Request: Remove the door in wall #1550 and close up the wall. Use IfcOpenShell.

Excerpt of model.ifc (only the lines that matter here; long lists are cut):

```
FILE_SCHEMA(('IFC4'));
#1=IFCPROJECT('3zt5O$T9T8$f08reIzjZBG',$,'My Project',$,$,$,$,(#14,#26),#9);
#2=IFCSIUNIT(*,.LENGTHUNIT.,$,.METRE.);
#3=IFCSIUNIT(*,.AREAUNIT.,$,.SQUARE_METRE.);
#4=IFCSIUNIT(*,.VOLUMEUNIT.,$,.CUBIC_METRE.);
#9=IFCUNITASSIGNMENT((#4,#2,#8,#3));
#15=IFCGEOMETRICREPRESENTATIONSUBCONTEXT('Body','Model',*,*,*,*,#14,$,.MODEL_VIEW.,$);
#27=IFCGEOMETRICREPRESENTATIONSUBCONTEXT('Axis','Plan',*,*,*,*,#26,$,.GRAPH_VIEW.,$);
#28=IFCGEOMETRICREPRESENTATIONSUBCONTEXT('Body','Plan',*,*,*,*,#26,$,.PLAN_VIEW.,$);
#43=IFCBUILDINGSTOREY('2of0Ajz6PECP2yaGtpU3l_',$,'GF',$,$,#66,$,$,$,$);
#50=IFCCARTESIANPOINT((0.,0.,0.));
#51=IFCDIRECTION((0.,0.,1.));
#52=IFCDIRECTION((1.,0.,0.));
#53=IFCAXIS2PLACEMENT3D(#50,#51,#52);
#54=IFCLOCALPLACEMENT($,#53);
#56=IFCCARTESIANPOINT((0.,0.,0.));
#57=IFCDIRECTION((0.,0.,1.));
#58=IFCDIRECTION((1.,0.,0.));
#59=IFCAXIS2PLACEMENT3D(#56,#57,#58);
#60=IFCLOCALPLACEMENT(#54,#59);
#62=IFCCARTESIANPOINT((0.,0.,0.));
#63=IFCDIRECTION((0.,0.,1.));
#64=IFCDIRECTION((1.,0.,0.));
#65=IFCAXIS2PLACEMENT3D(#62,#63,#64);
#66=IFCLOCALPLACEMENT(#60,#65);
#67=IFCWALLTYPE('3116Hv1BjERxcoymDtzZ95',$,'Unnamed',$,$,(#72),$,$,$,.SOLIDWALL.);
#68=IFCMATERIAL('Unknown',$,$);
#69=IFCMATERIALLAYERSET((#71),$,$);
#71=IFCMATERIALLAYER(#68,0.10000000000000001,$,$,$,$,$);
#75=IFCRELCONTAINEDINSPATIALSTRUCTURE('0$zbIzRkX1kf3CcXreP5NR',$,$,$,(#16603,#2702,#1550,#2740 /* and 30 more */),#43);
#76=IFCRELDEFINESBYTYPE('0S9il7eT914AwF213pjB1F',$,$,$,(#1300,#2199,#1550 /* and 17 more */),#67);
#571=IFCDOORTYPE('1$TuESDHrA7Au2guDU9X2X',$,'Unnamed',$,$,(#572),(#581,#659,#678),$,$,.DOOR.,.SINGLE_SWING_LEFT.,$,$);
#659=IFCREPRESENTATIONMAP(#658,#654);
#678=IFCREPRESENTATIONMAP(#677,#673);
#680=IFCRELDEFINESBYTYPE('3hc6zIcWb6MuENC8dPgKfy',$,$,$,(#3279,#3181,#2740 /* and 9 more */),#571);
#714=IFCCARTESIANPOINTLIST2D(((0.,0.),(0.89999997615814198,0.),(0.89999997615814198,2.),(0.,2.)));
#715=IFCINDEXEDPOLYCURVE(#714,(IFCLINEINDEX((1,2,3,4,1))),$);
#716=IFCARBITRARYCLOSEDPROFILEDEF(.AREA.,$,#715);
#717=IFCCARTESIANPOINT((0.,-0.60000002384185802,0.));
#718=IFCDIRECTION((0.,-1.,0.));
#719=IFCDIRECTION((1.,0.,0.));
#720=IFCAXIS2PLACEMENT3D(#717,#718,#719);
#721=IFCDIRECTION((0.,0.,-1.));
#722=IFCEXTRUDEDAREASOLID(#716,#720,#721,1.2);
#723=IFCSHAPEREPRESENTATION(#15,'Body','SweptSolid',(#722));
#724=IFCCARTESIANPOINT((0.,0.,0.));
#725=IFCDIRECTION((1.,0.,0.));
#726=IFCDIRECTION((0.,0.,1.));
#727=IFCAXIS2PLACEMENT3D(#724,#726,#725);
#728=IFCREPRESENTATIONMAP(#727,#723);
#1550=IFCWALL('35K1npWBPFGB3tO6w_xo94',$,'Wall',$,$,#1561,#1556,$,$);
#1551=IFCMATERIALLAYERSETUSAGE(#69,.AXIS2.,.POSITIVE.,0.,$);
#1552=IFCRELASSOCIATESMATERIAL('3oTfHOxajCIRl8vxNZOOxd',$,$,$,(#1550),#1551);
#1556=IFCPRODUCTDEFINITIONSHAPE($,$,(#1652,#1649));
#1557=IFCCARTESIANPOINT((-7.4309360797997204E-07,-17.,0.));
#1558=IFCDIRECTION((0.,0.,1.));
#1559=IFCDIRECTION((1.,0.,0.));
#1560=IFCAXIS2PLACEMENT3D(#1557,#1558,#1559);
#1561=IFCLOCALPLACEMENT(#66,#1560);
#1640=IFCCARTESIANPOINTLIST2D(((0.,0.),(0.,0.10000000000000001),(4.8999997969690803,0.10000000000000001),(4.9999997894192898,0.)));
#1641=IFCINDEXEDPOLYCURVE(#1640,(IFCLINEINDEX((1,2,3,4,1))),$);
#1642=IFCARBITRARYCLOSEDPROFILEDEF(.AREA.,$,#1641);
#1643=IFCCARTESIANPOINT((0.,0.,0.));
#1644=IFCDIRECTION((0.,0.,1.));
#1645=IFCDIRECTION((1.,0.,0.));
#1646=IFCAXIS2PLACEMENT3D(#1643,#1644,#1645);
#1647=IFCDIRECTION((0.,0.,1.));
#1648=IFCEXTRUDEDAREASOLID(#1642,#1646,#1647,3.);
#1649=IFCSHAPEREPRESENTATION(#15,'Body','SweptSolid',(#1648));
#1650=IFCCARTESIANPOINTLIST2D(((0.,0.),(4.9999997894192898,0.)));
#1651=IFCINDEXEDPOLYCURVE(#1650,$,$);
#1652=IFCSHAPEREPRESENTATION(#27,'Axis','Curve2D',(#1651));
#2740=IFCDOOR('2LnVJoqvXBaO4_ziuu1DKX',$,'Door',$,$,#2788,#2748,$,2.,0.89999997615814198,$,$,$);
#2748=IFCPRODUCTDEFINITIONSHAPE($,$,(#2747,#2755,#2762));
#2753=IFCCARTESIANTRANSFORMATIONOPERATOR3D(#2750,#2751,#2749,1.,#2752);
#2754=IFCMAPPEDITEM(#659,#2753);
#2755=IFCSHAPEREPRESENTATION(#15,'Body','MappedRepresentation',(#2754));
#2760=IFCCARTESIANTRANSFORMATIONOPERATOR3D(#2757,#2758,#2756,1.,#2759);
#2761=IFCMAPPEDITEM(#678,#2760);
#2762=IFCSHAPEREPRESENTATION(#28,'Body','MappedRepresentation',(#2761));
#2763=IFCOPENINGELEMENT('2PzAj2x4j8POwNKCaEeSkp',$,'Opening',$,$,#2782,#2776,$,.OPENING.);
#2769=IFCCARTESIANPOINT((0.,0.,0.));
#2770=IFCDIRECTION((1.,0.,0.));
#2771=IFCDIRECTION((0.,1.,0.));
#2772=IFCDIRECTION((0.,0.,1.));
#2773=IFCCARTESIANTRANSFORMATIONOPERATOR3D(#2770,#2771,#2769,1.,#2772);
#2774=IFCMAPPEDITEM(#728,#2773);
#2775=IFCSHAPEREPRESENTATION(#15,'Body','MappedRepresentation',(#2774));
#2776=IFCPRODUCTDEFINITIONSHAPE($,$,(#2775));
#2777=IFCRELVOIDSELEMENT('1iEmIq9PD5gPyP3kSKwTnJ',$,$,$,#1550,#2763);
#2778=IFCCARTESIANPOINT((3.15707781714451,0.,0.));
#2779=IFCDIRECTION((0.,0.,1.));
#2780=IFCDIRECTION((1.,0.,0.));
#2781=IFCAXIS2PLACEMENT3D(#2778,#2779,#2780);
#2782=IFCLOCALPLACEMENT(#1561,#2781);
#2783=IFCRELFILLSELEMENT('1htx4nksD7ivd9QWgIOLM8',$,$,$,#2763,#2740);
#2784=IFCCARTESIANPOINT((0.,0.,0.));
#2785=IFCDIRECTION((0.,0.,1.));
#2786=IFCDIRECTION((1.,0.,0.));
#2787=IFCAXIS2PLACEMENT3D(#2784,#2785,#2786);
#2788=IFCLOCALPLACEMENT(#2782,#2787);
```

```python
import ifcopenshell
import ifcopenshell.api.feature
import ifcopenshell.api.root
import ifcopenshell.geom
import ifcopenshell.util.shape

model = ifcopenshell.open("model.ifc")
settings = ifcopenshell.geom.settings()


def volume(element):
    """Net volume in cubic metres, openings subtracted."""
    shape = ifcopenshell.geom.create_shape(settings, element)
    return ifcopenshell.util.shape.get_volume(shape.geometry)


door = model.by_guid("2LnVJoqvXBaO4_ziuu1DKX")
opening = door.FillsVoids[0].RelatingOpeningElement
wall = opening.VoidsElements[0].RelatingBuildingElement
before = volume(wall)

ifcopenshell.api.root.remove_product(model, product=door)
ifcopenshell.api.feature.remove_feature(model, feature=opening)

after = volume(wall)

print(f"wall volume {before:.3f} -> {after:.3f} m3")

model.write("model_edited.ifc")
```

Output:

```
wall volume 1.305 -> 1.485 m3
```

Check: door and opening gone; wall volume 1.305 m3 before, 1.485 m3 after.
